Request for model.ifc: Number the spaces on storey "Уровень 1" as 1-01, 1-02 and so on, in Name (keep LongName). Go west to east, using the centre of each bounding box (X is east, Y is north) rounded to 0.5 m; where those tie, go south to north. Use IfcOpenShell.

First a look at what the model holds.

```python
import ifcopenshell
import ifcopenshell.util.element
import ifcopenshell.util.placement

model = ifcopenshell.open("model.ifc")
print(model.schema)
storey = next(s for s in model.by_type("IfcBuildingStorey") if s.Name == "Уровень 1")
spaces = [e for e in ifcopenshell.util.element.get_decomposition(storey) if e.is_a("IfcSpace")]
for e in sorted(spaces, key=lambda e: e.id()):
    origin = ifcopenshell.util.placement.get_local_placement(e.ObjectPlacement)[:3, 3]
    print(e.id(), e.Name, e.LongName, origin.round(2) + 0.0, sep=" | ")
```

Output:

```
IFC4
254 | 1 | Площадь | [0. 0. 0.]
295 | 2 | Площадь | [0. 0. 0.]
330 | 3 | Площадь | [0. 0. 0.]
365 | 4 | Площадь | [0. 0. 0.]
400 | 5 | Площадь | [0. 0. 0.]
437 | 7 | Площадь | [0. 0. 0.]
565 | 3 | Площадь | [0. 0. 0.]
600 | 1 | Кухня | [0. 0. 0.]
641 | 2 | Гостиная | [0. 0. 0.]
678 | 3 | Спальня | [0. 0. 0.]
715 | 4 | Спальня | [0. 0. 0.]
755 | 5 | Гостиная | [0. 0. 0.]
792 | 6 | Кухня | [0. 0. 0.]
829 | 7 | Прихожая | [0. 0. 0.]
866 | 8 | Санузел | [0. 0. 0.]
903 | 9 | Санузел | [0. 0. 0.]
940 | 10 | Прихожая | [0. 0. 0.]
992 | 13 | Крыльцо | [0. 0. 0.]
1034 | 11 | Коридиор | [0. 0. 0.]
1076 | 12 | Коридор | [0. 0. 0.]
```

```python
import ifcopenshell
import ifcopenshell.geom
import ifcopenshell.util.element
import ifcopenshell.util.shape

model = ifcopenshell.open("model.ifc")
settings = ifcopenshell.geom.settings()
settings.set("use-world-coords", True)


def centre(element):
    shape = ifcopenshell.geom.create_shape(settings, element)
    return ifcopenshell.util.shape.get_bbox_centroid(shape.geometry)


storey = next(s for s in model.by_type("IfcBuildingStorey") if s.Name == "Уровень 1")
spaces = [e for e in ifcopenshell.util.element.get_decomposition(storey) if e.is_a("IfcSpace")]

# Insertion points can sit at a corner or the storey origin, so sort by the geometry (in metres).
centres = {e: centre(e) for e in spaces}
spaces.sort(key=lambda e: (round(centres[e][0] / 0.5), centres[e][1]))

for i, e in enumerate(spaces, start=1):
    number = f"1-{i:02d}"
    e.Name = number
    print(e.id(), number)

model.write("model_edited.ifc")
```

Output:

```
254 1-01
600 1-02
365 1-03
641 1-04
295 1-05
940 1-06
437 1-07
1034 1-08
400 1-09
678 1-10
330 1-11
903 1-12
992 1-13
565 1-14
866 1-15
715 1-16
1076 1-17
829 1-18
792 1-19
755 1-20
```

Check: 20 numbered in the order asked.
